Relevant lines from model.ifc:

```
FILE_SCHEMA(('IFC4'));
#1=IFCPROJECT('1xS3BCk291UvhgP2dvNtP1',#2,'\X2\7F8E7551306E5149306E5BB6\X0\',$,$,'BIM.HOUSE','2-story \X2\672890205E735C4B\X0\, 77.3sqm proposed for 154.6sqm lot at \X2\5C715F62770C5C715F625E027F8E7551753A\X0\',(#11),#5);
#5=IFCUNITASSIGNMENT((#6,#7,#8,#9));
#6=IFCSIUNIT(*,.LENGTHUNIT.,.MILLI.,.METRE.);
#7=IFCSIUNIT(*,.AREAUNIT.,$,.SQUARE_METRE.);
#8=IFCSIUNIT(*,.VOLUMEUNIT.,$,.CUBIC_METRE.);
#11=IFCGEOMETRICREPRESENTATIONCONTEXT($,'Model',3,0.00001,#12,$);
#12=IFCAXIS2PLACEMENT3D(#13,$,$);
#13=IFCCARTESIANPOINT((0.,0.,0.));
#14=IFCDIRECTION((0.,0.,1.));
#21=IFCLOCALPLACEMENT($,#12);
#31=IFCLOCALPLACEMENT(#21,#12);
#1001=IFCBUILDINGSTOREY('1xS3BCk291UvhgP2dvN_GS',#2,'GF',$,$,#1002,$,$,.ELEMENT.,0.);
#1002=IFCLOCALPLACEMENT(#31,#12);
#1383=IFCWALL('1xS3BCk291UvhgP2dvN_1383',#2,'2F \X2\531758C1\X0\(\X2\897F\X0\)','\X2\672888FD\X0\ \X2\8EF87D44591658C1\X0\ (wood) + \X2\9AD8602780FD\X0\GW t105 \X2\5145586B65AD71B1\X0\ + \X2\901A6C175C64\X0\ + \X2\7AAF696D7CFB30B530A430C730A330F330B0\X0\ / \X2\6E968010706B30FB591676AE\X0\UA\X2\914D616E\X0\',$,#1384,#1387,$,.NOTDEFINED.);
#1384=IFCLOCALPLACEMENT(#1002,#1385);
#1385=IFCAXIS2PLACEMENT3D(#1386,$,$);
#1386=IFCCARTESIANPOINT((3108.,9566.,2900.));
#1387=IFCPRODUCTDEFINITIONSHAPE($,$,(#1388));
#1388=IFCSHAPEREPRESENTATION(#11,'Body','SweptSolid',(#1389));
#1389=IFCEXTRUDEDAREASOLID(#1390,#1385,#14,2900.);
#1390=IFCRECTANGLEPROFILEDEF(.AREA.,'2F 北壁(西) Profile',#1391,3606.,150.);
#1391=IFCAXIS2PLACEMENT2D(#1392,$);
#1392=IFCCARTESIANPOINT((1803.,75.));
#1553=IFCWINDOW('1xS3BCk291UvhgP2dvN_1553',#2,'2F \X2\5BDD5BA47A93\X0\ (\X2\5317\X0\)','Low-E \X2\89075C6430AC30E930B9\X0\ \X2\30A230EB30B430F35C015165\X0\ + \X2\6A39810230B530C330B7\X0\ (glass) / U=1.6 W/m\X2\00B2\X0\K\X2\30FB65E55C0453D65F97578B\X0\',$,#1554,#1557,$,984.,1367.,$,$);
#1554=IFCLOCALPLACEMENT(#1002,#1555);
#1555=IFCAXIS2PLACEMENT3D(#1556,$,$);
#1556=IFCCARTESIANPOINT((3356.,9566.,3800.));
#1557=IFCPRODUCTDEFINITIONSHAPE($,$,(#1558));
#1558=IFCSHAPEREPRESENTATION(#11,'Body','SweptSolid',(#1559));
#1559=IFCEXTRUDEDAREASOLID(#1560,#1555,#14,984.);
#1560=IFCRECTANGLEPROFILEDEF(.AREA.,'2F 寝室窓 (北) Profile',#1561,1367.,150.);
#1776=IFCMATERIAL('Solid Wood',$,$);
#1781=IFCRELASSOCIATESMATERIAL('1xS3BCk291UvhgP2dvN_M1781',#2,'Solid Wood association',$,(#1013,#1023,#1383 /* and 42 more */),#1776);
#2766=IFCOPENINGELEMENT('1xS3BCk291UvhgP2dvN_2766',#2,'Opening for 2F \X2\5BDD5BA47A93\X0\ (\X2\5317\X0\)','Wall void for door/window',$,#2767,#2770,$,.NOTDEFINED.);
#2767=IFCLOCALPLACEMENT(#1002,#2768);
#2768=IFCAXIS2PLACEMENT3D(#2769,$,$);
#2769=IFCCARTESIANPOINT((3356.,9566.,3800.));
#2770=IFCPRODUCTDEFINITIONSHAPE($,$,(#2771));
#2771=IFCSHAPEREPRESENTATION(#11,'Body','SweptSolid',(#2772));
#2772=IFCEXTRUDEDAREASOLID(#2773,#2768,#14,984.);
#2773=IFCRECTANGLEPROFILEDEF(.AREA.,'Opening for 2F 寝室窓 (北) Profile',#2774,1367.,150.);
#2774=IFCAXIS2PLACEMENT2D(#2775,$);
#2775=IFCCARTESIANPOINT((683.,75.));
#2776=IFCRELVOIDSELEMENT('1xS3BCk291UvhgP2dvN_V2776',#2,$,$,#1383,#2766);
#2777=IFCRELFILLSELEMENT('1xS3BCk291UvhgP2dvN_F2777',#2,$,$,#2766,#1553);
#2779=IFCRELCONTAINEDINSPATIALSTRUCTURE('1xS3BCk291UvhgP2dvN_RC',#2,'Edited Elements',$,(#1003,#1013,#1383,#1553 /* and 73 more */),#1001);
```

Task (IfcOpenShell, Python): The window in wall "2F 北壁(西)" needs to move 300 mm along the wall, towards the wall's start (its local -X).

```python
import ifcopenshell
import ifcopenshell.api.geometry
import ifcopenshell.util.placement

model = ifcopenshell.open("model.ifc")

window = model.by_guid("1xS3BCk291UvhgP2dvN_1553")
opening = window.FillsVoids[0].RelatingOpeningElement
wall = opening.VoidsElements[0].RelatingBuildingElement

wall_matrix = ifcopenshell.util.placement.get_local_placement(wall.ObjectPlacement)
shift = wall_matrix[:3, 0] * -300.0
before = ifcopenshell.util.placement.get_local_placement(window.ObjectPlacement)[:3, 3].copy()

# The window is not placed relative to its opening, so move both.
for product in (opening, window):
    matrix = ifcopenshell.util.placement.get_local_placement(product.ObjectPlacement)
    matrix[:3, 3] += shift
    ifcopenshell.api.geometry.edit_object_placement(model, product=product, matrix=matrix, is_si=False)

after = ifcopenshell.util.placement.get_local_placement(window.ObjectPlacement)[:3, 3]
print("window moved by", (after - before).round(3) + 0.0)

model.write("model-out.ifc")
```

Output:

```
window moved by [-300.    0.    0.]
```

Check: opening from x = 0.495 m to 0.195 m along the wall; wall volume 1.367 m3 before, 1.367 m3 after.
